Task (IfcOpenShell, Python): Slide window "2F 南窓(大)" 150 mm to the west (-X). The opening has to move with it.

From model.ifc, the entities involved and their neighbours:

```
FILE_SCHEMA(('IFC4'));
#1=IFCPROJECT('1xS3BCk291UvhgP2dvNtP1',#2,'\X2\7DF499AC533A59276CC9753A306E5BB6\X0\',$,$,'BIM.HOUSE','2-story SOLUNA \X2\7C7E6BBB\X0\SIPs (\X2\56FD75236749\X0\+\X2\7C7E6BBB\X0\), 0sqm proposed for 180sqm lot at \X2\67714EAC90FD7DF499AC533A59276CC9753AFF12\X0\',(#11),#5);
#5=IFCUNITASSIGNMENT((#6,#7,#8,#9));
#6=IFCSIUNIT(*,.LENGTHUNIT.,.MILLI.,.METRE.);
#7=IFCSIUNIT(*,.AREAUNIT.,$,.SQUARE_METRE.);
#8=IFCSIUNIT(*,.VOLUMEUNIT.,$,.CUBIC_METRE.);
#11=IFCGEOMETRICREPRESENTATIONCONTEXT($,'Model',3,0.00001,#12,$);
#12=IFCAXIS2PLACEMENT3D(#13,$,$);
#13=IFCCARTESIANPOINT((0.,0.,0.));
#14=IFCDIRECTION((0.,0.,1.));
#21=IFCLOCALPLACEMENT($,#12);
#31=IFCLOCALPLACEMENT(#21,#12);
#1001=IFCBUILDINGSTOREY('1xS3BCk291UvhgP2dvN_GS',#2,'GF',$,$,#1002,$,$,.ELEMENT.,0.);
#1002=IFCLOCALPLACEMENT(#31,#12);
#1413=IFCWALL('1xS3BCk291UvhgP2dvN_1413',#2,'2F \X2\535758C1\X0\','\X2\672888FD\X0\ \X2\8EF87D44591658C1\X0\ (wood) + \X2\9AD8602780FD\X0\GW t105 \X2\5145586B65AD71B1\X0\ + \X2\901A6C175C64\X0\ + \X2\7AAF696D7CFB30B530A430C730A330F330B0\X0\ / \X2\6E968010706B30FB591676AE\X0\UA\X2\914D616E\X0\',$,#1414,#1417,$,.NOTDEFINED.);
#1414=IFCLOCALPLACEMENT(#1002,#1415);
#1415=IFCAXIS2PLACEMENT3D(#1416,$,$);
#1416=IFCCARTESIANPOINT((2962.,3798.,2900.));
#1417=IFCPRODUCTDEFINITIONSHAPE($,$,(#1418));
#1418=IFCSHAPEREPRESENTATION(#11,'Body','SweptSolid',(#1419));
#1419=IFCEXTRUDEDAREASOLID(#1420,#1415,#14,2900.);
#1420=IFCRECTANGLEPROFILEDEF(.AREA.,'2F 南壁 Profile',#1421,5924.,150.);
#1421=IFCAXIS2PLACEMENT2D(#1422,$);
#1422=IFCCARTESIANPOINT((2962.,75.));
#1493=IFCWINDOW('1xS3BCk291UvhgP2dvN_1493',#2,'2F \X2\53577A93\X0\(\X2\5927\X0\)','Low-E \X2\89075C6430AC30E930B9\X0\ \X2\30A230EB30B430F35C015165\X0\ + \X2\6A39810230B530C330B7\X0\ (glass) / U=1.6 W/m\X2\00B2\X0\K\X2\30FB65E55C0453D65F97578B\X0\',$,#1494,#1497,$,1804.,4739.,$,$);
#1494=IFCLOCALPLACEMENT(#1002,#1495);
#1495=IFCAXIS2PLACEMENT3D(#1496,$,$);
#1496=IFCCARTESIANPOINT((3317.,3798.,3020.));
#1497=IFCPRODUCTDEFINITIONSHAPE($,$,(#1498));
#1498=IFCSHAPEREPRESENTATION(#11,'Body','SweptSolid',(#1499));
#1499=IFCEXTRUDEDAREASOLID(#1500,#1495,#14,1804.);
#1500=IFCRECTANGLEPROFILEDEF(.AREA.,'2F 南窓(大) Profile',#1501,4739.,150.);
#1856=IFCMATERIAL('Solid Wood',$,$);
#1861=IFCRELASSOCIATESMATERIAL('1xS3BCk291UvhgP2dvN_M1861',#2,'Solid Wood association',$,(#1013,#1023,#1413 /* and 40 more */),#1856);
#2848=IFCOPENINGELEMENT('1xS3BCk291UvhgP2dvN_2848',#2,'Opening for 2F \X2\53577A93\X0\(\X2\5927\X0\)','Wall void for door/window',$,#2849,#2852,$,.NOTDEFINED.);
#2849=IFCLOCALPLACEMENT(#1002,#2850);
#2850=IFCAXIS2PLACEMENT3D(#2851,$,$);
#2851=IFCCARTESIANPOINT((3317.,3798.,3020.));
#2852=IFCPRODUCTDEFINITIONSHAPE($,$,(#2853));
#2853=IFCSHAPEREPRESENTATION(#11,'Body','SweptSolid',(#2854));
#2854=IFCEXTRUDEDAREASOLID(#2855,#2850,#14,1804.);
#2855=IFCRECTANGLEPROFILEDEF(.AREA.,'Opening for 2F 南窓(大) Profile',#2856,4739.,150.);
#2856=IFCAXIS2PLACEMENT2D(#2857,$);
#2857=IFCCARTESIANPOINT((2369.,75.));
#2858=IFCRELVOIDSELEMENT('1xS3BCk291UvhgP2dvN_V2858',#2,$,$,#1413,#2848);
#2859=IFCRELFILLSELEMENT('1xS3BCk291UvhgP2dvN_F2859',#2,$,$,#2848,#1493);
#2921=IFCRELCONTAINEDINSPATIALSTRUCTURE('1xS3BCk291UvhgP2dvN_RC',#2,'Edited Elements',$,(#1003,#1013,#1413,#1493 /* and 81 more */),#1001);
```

```python
import ifcopenshell
import ifcopenshell.api.geometry
import ifcopenshell.util.placement
import ifcopenshell.util.unit

model = ifcopenshell.open("model.ifc")
unit_scale = ifcopenshell.util.unit.calculate_unit_scale(model)

window = model.by_guid("1xS3BCk291UvhgP2dvN_1493")
opening = window.FillsVoids[0].RelatingOpeningElement
wall = opening.VoidsElements[0].RelatingBuildingElement

wall_matrix = ifcopenshell.util.placement.get_local_placement(wall.ObjectPlacement)
shift = wall_matrix[:3, 0] * -0.15 / unit_scale
before = ifcopenshell.util.placement.get_local_placement(window.ObjectPlacement)[:3, 3].copy()

# The window is not placed relative to its opening, so move both.
for product in (opening, window):
    matrix = ifcopenshell.util.placement.get_local_placement(product.ObjectPlacement)
    matrix[:3, 3] += shift
    ifcopenshell.api.geometry.edit_object_placement(model, product=product, matrix=matrix, is_si=False)

after = ifcopenshell.util.placement.get_local_placement(window.ObjectPlacement)[:3, 3]
print("window moved by", (after - before).round(3) + 0.0)

model.write("model-out.ifc")
```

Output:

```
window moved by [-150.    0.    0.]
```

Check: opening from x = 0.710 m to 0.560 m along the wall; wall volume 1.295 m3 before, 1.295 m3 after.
